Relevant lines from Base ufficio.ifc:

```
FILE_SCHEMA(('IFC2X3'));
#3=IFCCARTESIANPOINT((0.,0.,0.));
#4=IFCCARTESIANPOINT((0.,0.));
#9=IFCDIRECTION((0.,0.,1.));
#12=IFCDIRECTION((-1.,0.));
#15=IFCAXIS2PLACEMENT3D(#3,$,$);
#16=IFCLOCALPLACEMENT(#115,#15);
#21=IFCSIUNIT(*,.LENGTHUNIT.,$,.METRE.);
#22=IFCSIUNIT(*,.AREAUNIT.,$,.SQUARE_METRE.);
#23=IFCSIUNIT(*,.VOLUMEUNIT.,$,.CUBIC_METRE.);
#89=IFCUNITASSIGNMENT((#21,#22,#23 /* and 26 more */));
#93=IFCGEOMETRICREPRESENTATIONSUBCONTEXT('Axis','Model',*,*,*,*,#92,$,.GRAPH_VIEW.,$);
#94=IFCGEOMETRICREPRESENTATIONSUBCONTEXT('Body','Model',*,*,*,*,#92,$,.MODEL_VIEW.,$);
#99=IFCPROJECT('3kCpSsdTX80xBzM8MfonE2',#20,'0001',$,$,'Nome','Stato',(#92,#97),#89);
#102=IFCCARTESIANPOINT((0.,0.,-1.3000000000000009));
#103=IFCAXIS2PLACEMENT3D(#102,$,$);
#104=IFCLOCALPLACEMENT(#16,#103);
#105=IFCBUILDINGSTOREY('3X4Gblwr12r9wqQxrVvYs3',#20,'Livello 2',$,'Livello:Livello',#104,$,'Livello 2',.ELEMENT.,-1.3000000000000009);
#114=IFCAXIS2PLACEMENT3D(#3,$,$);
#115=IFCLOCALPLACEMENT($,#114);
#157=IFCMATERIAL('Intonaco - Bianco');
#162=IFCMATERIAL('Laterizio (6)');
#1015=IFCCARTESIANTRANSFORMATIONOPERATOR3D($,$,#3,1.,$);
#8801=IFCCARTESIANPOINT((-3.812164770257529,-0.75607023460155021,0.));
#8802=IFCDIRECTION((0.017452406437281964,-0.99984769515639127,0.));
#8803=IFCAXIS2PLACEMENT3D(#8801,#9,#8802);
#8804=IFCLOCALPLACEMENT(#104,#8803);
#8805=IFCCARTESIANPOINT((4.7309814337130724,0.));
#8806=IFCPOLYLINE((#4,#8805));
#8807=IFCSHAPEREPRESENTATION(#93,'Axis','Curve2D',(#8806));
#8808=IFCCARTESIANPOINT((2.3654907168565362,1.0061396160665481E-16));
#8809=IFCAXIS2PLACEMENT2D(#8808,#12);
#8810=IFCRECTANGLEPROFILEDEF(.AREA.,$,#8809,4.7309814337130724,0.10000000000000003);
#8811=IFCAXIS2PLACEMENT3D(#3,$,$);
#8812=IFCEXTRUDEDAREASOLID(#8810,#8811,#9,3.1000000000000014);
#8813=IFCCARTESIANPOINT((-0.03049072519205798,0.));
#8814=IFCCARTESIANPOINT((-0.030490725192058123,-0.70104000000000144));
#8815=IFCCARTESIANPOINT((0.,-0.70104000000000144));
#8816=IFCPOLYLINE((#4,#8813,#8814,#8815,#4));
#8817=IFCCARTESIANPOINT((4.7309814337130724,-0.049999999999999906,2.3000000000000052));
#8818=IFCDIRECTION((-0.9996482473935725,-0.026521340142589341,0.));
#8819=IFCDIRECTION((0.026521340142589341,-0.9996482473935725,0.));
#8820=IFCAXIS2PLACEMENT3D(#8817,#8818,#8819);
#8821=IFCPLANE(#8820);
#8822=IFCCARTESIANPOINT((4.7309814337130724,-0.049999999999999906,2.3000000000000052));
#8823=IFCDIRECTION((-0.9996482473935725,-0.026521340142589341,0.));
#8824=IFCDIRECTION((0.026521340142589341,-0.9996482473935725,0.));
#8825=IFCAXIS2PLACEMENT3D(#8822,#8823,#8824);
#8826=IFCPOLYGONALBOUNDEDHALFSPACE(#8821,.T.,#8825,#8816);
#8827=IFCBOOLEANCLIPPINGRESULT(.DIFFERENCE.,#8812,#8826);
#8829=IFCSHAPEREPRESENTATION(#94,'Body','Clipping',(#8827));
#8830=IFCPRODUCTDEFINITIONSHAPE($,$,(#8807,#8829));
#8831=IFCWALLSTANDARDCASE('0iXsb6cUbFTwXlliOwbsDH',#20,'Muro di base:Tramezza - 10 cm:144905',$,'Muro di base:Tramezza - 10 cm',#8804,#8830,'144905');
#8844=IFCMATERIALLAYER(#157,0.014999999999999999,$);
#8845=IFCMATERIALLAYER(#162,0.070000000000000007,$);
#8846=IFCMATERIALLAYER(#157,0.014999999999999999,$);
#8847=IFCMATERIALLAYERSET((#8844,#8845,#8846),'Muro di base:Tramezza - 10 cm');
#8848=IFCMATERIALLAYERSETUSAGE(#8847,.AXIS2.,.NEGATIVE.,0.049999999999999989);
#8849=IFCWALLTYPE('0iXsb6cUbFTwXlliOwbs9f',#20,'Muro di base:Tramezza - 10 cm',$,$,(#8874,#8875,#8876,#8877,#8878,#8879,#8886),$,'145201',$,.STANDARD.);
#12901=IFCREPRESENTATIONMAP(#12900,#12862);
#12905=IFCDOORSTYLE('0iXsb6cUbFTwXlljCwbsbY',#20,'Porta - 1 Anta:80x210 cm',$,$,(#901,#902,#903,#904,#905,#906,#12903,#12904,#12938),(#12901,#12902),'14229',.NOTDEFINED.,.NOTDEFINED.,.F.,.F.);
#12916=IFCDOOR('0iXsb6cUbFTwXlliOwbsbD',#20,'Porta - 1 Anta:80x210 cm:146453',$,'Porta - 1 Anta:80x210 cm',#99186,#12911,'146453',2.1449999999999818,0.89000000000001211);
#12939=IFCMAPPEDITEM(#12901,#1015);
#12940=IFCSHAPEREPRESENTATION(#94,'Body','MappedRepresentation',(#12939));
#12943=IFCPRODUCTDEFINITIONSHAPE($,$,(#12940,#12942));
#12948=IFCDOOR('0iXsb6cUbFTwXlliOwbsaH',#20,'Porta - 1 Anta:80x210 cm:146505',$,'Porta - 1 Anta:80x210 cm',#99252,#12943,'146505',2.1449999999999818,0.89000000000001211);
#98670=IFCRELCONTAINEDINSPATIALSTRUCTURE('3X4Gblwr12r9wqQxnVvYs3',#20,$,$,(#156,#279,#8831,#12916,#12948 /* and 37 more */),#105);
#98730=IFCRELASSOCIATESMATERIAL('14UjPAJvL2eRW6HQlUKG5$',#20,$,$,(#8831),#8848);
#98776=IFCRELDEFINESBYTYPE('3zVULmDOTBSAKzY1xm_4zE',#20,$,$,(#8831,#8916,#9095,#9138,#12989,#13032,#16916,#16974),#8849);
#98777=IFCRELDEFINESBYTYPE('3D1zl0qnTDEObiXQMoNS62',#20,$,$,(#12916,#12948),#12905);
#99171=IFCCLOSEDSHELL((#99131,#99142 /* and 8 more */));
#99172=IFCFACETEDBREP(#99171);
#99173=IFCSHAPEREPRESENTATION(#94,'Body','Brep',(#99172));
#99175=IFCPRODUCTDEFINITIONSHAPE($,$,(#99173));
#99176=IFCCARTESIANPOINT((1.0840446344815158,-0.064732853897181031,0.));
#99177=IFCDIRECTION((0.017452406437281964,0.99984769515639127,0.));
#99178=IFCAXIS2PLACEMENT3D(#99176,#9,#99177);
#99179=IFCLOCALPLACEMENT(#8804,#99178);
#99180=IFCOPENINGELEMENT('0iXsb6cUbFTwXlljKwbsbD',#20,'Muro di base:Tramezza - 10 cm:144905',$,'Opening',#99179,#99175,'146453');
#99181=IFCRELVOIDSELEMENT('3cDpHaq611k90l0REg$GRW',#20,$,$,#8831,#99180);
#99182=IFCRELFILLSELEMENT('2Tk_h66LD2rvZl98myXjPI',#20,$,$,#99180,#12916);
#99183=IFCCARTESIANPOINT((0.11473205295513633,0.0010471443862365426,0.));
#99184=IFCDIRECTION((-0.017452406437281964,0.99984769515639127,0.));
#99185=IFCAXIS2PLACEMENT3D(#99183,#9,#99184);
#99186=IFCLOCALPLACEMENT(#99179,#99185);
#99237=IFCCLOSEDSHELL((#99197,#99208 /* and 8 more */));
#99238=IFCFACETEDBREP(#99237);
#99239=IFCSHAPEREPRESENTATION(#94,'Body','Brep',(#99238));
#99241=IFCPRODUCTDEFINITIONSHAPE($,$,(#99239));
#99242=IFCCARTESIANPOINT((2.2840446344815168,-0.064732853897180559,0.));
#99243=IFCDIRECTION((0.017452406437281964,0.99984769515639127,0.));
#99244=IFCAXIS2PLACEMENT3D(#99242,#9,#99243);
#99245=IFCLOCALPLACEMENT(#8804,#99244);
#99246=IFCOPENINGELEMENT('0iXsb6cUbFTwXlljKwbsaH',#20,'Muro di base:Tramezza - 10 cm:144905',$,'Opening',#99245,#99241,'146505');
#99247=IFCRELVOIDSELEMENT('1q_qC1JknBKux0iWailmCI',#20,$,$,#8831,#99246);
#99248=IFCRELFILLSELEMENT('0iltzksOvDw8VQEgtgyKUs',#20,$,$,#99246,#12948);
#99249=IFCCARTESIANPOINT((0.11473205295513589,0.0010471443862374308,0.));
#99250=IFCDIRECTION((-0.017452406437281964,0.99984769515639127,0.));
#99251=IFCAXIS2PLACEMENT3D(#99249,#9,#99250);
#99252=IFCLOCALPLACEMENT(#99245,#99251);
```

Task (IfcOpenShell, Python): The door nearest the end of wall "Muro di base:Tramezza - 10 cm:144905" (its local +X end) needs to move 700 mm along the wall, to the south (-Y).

```python
import ifcopenshell
import ifcopenshell.api.geometry
import ifcopenshell.util.placement

model = ifcopenshell.open("Base ufficio.ifc")

door = model.by_id(12948)
opening = door.FillsVoids[0].RelatingOpeningElement
wall = opening.VoidsElements[0].RelatingBuildingElement

wall_matrix = ifcopenshell.util.placement.get_local_placement(wall.ObjectPlacement)
shift = wall_matrix[:3, 0] * 0.7
before = ifcopenshell.util.placement.get_local_placement(door.ObjectPlacement)[:3, 3].copy()

# The door is placed relative to its opening, so it follows when the opening moves.
matrix = ifcopenshell.util.placement.get_local_placement(opening.ObjectPlacement)
matrix[:3, 3] += shift
ifcopenshell.api.geometry.edit_object_placement(
    model, product=opening, matrix=matrix, is_si=False, should_transform_children=True
)

after = ifcopenshell.util.placement.get_local_placement(door.ObjectPlacement)[:3, 3]
print("door moved by", (after - before).round(3) + 0.0)

model.write("Base ufficio-out.ifc")
```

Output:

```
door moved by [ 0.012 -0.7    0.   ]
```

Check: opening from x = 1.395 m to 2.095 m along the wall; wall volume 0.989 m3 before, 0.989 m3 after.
